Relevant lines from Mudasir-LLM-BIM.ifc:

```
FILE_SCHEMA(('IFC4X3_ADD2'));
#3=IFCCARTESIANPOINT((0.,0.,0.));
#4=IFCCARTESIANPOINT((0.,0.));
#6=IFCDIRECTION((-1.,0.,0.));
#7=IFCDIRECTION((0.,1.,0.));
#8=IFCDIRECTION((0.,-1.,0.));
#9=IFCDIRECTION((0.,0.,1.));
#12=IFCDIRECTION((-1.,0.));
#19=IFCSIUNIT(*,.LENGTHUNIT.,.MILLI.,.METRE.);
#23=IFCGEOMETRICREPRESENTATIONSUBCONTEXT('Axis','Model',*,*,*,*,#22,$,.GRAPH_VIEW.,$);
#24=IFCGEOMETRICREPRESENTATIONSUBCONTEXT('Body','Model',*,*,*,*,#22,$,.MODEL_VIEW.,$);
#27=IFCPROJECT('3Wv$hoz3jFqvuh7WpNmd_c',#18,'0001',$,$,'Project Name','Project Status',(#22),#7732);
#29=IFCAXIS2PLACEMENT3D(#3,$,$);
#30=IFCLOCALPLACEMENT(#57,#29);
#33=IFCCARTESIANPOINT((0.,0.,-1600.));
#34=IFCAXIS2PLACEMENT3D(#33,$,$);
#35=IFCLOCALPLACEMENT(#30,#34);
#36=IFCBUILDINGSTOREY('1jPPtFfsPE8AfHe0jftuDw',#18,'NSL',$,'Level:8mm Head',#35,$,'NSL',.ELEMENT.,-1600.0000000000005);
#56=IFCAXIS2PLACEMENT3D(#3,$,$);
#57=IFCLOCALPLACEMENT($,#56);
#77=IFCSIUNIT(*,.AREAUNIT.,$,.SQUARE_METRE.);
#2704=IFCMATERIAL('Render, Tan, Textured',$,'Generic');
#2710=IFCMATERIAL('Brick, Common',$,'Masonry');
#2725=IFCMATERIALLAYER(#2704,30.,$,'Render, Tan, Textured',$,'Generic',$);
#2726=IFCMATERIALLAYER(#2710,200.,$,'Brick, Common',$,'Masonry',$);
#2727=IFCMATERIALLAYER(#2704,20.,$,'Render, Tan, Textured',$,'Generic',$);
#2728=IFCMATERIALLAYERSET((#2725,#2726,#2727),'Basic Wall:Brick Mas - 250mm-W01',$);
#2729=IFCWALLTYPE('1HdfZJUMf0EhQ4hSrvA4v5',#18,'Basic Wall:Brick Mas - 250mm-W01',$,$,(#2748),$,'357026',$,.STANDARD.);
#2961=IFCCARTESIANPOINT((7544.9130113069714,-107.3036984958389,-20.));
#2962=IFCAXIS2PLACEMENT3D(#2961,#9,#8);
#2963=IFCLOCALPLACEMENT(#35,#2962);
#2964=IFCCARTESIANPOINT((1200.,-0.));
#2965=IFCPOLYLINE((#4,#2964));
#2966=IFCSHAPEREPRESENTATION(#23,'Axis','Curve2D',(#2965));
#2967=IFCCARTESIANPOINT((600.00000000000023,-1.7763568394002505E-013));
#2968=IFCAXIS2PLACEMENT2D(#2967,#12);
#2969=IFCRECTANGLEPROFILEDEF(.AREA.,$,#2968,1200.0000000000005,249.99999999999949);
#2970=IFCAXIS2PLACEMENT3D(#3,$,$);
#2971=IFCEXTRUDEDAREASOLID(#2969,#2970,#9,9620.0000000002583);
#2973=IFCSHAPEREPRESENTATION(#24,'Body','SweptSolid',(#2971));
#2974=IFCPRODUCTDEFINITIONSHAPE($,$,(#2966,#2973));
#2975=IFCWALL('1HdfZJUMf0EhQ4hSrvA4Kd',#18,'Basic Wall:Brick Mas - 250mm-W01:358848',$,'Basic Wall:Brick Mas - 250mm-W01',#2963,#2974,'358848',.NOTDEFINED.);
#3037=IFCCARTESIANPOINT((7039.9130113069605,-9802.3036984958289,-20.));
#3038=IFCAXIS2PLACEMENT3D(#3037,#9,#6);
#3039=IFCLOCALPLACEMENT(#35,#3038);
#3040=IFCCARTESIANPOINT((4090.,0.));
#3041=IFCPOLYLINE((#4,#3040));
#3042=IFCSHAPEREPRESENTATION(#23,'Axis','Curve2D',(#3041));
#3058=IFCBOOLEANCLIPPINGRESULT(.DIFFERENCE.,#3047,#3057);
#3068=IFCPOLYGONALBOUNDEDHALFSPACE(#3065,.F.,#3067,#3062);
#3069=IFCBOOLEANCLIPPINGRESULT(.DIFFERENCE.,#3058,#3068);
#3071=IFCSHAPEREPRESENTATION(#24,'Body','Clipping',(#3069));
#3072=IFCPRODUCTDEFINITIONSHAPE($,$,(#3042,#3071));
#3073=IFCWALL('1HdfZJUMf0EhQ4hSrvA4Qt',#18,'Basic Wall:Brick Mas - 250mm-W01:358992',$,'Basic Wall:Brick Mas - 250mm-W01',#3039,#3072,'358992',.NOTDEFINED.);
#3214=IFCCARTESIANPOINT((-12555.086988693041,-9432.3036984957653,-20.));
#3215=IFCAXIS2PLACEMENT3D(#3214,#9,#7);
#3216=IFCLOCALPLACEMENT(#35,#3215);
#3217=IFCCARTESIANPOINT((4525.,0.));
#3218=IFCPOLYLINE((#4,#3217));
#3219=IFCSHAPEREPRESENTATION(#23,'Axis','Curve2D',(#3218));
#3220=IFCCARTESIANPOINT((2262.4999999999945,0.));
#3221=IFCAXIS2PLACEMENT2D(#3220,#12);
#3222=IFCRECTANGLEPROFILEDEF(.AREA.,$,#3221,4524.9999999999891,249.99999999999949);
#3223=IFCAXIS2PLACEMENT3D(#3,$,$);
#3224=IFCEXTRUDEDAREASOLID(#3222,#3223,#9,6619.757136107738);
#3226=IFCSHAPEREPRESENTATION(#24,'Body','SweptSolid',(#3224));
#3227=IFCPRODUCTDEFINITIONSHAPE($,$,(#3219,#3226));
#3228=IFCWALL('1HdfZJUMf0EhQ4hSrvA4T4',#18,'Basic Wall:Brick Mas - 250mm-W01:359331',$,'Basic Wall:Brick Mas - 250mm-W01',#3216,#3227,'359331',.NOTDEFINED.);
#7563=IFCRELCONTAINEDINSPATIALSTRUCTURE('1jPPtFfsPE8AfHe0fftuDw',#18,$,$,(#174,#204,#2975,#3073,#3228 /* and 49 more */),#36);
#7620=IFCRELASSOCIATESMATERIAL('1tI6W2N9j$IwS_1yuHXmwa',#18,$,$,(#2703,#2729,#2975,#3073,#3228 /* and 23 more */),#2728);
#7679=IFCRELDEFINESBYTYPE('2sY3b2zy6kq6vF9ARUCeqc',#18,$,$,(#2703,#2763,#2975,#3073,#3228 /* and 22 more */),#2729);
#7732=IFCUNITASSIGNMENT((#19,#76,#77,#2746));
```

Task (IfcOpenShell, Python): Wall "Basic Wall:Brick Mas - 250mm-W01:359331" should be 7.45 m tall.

```python
import ifcopenshell
import ifcopenshell.geom
import ifcopenshell.util.representation
import ifcopenshell.util.shape

model = ifcopenshell.open("Mudasir-LLM-BIM.ifc")
settings = ifcopenshell.geom.settings()


def volume(element):
    """Net volume in cubic metres, openings subtracted."""
    shape = ifcopenshell.geom.create_shape(settings, element)
    return ifcopenshell.util.shape.get_volume(shape.geometry)


wall = model.by_guid("1HdfZJUMf0EhQ4hSrvA4T4")
before = volume(wall)

body = ifcopenshell.util.representation.get_representation(wall, "Model", "Body")
solid = body.Items[0]
old_height = solid.Depth
solid.Depth = 7450.0
after = volume(wall)

print(f"height {old_height:g} -> {solid.Depth:g}, volume {before:.3f} -> {after:.3f} m3")

model.write("Mudasir-LLM-BIM_edited.ifc")
```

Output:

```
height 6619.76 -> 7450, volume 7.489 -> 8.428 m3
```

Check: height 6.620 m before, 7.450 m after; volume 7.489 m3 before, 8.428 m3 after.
